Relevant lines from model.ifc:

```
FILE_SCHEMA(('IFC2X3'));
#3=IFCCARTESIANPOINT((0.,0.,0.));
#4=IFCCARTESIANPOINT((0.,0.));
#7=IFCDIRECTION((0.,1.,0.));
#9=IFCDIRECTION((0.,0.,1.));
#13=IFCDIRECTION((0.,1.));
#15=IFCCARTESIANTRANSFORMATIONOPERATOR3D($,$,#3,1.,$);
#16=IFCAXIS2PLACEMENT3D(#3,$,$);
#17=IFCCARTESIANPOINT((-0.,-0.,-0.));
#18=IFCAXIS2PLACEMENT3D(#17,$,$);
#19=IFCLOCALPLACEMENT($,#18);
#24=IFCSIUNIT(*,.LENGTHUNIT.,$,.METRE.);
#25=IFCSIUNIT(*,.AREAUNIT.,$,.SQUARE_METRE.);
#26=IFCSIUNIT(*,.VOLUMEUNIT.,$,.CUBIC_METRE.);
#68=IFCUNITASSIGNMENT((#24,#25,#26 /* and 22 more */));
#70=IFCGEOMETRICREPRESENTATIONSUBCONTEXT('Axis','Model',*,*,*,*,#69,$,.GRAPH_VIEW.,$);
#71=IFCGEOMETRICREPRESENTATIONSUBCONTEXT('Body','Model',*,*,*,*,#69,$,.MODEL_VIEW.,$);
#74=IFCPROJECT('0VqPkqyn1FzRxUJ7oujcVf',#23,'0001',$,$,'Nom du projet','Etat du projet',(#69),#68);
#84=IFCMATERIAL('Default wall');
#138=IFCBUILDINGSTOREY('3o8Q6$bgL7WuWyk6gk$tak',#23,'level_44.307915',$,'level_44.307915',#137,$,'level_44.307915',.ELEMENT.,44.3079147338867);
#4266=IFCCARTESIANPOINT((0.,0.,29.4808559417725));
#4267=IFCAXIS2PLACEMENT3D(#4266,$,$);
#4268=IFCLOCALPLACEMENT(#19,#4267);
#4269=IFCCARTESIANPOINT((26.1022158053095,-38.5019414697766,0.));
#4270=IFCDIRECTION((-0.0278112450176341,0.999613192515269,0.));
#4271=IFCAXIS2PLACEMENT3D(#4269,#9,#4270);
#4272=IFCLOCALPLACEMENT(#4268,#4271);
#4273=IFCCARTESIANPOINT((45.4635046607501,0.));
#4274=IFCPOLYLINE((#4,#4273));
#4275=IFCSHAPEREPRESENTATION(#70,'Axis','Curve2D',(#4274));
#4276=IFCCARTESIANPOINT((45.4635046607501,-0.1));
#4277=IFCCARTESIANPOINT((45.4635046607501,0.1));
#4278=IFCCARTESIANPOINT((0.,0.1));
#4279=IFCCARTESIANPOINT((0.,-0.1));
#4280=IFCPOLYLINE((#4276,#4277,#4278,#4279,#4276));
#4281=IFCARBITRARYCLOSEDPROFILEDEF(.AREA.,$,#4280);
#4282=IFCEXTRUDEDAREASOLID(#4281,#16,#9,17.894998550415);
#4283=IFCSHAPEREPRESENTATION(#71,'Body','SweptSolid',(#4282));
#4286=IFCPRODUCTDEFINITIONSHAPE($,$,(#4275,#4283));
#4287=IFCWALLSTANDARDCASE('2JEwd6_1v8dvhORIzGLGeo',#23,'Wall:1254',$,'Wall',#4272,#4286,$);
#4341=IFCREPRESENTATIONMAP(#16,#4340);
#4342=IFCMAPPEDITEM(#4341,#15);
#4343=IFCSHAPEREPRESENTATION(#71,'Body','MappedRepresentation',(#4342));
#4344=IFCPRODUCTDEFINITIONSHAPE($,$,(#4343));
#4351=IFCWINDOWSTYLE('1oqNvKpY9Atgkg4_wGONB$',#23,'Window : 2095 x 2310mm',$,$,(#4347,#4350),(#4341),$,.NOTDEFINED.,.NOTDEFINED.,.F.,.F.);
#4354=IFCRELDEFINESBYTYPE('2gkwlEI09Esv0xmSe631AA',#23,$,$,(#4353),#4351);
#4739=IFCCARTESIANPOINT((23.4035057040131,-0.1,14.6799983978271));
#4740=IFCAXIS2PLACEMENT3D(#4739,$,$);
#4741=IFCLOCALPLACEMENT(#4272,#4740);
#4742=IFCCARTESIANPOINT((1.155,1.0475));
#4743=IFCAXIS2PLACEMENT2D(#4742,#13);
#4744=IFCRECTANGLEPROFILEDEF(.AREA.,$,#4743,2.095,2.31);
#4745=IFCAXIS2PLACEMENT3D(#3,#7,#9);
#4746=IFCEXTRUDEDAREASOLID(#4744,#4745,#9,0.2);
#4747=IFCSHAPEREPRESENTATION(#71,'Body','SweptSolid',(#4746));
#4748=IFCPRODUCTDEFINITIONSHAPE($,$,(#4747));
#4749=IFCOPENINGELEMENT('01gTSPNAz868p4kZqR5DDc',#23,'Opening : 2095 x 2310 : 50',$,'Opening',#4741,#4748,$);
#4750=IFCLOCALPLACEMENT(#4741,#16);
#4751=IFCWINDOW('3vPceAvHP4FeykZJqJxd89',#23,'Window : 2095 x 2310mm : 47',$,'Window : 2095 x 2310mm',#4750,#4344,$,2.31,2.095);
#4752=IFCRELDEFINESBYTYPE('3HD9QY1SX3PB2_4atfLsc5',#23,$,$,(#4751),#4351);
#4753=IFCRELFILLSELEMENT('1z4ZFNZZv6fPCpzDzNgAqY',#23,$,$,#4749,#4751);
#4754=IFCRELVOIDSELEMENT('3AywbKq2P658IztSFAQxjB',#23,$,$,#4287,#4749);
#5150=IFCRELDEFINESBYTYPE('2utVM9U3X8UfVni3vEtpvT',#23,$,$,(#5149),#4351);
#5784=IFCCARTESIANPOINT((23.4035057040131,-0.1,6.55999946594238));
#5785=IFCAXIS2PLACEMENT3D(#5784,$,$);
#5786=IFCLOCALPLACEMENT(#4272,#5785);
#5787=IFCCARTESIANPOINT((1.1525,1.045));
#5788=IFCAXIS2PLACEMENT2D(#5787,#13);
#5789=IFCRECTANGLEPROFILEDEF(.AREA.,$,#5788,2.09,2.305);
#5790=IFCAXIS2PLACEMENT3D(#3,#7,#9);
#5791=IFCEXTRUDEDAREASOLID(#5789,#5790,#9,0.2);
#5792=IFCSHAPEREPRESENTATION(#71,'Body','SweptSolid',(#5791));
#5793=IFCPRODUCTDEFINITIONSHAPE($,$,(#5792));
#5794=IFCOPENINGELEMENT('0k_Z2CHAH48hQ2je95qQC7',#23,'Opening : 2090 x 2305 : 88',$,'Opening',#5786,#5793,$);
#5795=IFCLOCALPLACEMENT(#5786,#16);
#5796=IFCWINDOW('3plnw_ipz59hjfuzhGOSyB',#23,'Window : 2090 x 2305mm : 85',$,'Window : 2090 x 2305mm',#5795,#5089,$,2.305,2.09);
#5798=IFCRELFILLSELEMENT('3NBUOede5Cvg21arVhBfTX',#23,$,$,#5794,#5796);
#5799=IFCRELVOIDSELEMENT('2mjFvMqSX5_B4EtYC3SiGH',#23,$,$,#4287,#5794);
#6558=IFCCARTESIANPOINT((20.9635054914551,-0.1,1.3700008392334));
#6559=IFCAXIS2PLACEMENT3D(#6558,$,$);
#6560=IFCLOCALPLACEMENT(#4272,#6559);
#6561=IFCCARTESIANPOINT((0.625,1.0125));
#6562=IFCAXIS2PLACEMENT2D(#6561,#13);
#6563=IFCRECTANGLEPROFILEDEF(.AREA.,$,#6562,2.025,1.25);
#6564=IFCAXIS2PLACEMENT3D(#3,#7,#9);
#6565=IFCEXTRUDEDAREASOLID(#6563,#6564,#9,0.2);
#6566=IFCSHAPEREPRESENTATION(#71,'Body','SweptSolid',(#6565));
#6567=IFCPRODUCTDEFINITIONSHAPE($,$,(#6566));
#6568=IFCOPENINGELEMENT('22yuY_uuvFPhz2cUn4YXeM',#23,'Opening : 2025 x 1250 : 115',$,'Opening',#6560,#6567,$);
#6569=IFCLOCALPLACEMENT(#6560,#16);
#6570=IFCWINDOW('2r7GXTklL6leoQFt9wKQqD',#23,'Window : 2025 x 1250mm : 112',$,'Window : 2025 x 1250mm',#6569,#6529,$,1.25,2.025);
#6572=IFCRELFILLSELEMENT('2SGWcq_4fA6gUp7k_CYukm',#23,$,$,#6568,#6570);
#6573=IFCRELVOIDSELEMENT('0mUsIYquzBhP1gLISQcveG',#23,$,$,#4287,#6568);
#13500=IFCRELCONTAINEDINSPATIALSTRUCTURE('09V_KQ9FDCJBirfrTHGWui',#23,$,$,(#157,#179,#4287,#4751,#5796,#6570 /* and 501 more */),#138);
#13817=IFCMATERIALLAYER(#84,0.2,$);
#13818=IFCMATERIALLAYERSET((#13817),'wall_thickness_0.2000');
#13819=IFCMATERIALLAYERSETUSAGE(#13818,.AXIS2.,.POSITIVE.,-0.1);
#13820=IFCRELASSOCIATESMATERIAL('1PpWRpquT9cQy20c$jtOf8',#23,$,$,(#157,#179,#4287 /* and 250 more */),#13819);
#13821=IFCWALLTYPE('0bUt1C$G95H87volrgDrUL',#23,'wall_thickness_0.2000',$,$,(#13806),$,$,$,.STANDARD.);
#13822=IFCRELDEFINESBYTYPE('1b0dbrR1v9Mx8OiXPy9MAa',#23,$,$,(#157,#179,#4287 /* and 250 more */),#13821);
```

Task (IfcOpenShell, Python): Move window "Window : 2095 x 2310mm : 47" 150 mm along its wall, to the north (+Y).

```python
import ifcopenshell
import ifcopenshell.api.geometry
import ifcopenshell.util.placement
import ifcopenshell.util.unit

model = ifcopenshell.open("model.ifc")
unit_scale = ifcopenshell.util.unit.calculate_unit_scale(model)

window = model.by_guid("3vPceAvHP4FeykZJqJxd89")
opening = window.FillsVoids[0].RelatingOpeningElement
wall = opening.VoidsElements[0].RelatingBuildingElement

wall_matrix = ifcopenshell.util.placement.get_local_placement(wall.ObjectPlacement)
shift = wall_matrix[:3, 0] * 0.15 / unit_scale
before = ifcopenshell.util.placement.get_local_placement(window.ObjectPlacement)[:3, 3].copy()

# The window is placed relative to its opening, so it follows when the opening moves.
matrix = ifcopenshell.util.placement.get_local_placement(opening.ObjectPlacement)
matrix[:3, 3] += shift
ifcopenshell.api.geometry.edit_object_placement(
    model, product=opening, matrix=matrix, is_si=False, should_transform_children=True
)

after = ifcopenshell.util.placement.get_local_placement(window.ObjectPlacement)[:3, 3]
print("window moved by", (after - before).round(3) + 0.0)

model.write("model_edited.ifc")
```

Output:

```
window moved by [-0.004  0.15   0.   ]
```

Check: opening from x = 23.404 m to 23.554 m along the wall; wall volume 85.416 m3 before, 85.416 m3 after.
